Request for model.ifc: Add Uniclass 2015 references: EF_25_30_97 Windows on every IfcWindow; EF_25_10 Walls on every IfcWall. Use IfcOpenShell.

First a look at what the model holds.

```python
import ifcopenshell

model = ifcopenshell.open("model.ifc")
print(model.schema)
print("classifications:", [c.Name for c in model.by_type("IfcClassification")])
for ifc_class in ("IfcDoor", "IfcRoof", "IfcStair", "IfcWall", "IfcWindow"):
    print(ifc_class, len(model.by_type(ifc_class)))
```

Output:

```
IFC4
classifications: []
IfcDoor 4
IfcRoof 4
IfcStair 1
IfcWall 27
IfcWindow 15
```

```python
import ifcopenshell
import ifcopenshell.api.classification

model = ifcopenshell.open("model.ifc")

system = ifcopenshell.api.classification.add_classification(model, classification="Uniclass 2015")

codes = {
    "IfcWindow": ("EF_25_30_97", "Windows"),
    "IfcWall": ("EF_25_10", "Walls"),
}
for ifc_class, (code, name) in codes.items():
    products = model.by_type(ifc_class)
    ifcopenshell.api.classification.add_reference(
        model, products=products, classification=system, identification=code, name=name
    )
    print(code, len(products))

model.write("model_rev.ifc")
```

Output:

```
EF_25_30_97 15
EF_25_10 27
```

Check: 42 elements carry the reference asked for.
